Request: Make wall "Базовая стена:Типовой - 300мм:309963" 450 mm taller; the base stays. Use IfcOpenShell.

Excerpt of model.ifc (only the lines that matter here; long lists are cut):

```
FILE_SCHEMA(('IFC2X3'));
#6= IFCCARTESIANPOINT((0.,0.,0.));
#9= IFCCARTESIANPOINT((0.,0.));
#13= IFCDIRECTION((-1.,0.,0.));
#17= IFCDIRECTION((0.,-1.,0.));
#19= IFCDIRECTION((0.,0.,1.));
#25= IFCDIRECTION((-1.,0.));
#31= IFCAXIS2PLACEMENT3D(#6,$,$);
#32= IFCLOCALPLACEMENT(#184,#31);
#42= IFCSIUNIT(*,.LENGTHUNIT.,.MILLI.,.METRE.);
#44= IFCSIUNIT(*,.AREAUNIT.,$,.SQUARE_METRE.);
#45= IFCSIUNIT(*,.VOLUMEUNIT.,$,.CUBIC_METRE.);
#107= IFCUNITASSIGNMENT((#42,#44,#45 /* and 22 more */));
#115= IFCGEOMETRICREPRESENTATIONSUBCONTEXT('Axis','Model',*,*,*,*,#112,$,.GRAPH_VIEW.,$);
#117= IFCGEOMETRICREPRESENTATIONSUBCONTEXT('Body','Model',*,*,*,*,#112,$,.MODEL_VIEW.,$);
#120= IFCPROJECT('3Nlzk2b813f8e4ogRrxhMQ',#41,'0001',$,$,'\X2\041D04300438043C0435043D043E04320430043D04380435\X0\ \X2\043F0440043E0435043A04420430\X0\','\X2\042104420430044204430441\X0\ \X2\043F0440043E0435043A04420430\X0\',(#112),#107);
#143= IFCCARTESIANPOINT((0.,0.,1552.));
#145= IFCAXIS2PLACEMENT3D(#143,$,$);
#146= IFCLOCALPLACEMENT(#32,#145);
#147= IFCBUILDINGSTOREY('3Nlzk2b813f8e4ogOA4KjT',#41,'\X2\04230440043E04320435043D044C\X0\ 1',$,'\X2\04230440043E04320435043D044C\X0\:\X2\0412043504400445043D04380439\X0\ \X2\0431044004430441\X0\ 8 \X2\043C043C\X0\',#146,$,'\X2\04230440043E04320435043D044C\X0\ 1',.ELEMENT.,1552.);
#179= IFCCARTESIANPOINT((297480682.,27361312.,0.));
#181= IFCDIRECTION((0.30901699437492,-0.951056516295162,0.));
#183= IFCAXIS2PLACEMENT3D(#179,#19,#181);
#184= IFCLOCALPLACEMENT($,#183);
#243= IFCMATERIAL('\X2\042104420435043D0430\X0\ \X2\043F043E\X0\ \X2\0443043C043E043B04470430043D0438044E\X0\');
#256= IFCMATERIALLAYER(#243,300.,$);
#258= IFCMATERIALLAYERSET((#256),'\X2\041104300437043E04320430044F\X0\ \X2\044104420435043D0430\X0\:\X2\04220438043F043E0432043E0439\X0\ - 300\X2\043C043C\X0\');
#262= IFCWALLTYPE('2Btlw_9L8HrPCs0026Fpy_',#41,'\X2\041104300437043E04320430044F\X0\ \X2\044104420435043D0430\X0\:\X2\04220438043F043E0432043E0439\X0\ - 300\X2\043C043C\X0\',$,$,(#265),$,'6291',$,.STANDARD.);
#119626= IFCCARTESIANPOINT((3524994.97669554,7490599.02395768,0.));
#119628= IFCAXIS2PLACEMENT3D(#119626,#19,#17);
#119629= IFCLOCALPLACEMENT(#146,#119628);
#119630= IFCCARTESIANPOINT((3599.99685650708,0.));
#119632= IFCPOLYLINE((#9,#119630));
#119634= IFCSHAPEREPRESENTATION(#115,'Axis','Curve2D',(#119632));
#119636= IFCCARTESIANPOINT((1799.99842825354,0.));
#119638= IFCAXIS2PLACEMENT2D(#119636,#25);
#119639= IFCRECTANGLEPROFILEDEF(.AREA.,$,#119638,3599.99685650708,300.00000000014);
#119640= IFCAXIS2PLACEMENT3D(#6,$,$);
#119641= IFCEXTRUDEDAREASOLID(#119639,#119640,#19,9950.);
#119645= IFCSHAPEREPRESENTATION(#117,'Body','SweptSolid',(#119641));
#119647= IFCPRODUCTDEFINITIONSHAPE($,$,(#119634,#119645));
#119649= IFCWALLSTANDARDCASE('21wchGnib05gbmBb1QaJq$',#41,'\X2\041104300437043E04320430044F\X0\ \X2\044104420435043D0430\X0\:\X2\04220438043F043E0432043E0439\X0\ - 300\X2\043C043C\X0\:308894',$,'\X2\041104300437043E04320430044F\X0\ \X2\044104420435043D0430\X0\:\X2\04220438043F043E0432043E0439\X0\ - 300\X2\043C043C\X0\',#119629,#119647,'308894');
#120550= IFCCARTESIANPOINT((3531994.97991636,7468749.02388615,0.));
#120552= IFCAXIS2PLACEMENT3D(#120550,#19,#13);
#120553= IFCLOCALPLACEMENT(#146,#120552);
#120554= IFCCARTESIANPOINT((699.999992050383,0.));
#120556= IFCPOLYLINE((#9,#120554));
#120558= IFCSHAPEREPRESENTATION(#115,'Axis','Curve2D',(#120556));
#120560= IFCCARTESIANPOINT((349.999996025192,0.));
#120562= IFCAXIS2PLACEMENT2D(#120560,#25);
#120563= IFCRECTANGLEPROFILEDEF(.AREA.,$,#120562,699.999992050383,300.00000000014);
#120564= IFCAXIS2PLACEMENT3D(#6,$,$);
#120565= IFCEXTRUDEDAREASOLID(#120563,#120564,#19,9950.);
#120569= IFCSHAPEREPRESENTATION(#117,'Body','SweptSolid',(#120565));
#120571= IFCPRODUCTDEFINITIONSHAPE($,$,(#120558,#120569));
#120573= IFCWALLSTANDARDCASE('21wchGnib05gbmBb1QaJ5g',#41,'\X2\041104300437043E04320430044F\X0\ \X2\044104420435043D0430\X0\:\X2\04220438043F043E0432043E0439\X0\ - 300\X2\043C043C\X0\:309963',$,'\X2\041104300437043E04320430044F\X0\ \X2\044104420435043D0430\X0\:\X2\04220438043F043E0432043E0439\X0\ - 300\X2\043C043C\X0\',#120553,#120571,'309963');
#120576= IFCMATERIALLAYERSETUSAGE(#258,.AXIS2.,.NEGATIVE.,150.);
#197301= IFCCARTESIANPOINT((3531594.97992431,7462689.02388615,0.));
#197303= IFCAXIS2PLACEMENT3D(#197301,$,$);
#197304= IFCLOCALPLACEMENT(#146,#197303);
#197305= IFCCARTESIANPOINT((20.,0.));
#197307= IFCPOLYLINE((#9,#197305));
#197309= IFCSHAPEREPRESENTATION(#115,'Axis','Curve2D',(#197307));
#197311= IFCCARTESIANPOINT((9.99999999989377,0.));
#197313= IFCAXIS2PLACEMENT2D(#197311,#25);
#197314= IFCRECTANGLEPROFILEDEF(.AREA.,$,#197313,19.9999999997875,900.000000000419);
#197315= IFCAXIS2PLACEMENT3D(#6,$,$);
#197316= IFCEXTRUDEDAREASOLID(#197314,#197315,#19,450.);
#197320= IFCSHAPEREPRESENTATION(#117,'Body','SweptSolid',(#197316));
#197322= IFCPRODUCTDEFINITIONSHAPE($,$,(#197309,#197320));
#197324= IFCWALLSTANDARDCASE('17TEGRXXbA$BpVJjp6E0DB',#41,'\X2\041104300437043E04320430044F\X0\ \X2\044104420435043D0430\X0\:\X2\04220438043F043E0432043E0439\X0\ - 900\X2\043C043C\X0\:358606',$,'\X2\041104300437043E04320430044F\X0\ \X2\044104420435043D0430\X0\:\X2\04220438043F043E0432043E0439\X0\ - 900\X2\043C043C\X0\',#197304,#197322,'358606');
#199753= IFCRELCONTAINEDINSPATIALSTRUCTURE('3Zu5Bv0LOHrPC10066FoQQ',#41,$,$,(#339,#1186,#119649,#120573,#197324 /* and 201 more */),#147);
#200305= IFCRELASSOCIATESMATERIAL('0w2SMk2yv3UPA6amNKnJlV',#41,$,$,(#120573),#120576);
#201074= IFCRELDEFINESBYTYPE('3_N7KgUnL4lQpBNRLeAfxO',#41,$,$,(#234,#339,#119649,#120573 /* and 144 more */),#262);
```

```python
import ifcopenshell
import ifcopenshell.geom
import ifcopenshell.util.representation
import ifcopenshell.util.shape
import ifcopenshell.util.unit

model = ifcopenshell.open("model.ifc")
unit_scale = ifcopenshell.util.unit.calculate_unit_scale(model)
settings = ifcopenshell.geom.settings()


def volume(element):
    """Net volume in cubic metres, openings subtracted."""
    shape = ifcopenshell.geom.create_shape(settings, element)
    return ifcopenshell.util.shape.get_volume(shape.geometry)


wall = model.by_guid("21wchGnib05gbmBb1QaJ5g")
before = volume(wall)

body = ifcopenshell.util.representation.get_representation(wall, "Model", "Body")
solid = body.Items[0]
old_height = solid.Depth
solid.Depth += 0.45 / unit_scale
after = volume(wall)

print(f"height {old_height:g} -> {solid.Depth:g}, volume {before:.3f} -> {after:.3f} m3")

model.write("model_v2.ifc")
```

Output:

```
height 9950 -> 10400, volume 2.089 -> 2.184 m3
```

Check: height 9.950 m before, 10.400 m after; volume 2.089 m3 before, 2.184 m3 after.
